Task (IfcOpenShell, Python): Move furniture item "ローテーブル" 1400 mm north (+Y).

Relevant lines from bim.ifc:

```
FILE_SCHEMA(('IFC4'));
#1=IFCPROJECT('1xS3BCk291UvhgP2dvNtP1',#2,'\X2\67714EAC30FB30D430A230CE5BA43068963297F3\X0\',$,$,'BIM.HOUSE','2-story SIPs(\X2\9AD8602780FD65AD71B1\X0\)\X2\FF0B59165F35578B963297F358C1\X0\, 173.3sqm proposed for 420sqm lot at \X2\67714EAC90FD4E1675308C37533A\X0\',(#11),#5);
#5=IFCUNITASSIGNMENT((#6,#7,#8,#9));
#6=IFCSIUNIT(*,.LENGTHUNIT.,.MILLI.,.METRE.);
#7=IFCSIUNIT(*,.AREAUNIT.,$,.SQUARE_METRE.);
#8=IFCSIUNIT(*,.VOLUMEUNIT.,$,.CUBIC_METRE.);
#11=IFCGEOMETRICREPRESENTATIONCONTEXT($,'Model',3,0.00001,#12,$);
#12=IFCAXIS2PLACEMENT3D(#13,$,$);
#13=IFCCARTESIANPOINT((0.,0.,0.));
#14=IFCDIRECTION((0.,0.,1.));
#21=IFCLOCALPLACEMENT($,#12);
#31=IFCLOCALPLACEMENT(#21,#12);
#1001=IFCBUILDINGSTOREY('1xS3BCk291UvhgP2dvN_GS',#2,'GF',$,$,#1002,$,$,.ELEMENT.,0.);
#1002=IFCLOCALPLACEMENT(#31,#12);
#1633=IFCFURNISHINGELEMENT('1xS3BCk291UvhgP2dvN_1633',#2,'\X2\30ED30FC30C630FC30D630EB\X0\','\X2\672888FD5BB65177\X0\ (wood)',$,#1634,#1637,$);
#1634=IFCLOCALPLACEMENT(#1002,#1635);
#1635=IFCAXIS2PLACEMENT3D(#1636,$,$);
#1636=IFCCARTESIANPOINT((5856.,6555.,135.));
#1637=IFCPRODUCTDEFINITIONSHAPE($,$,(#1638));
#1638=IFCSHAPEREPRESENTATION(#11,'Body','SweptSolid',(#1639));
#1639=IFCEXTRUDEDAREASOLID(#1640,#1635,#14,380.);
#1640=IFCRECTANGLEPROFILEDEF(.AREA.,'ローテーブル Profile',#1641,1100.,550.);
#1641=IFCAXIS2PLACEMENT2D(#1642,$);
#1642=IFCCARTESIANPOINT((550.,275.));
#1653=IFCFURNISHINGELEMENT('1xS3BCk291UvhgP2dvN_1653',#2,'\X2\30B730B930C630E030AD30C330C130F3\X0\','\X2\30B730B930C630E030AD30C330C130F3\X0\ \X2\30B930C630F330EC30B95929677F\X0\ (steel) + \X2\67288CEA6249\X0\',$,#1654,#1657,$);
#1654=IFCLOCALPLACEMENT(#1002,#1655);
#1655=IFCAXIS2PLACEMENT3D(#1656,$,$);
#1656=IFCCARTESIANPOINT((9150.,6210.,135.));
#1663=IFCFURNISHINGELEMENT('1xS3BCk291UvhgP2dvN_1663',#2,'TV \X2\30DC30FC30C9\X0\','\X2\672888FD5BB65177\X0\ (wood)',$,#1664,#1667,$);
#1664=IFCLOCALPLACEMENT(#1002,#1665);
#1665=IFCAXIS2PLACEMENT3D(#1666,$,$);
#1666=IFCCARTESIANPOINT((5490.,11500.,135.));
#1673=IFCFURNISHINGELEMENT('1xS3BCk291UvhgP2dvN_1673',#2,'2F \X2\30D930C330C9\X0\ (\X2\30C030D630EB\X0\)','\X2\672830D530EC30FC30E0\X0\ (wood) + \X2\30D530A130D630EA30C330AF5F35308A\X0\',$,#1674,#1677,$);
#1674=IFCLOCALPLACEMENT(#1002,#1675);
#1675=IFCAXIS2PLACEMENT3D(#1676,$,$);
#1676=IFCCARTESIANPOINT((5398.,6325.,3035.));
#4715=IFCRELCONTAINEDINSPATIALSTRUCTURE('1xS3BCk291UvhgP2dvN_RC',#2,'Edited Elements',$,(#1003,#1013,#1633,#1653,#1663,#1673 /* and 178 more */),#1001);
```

```python
import ifcopenshell
import ifcopenshell.api.geometry
import ifcopenshell.util.placement

model = ifcopenshell.open("bim.ifc")

item = model.by_guid("1xS3BCk291UvhgP2dvN_1633")
matrix = ifcopenshell.util.placement.get_local_placement(item.ObjectPlacement)
matrix[1, 3] += 1400.0
ifcopenshell.api.geometry.edit_object_placement(model, product=item, matrix=matrix, is_si=False)

print(ifcopenshell.util.placement.get_local_placement(item.ObjectPlacement).round(3) + 0.0)

model.write("bim_edited.ifc")
```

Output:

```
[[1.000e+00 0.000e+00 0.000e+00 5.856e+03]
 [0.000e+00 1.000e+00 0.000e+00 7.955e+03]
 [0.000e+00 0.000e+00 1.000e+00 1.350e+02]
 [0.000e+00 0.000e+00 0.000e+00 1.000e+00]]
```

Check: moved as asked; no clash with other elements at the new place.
